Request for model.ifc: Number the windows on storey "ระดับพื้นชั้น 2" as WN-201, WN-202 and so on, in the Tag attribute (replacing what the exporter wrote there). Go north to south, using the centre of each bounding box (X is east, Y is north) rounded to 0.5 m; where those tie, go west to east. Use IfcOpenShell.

First a look at what the model holds.

```python
import ifcopenshell
import ifcopenshell.util.element
import ifcopenshell.util.placement

model = ifcopenshell.open("model.ifc")
print(model.schema)
storey = next(s for s in model.by_type("IfcBuildingStorey") if s.Name == "ระดับพื้นชั้น 2")
windows = [e for e in ifcopenshell.util.element.get_decomposition(storey) if e.is_a("IfcWindow")]
for e in sorted(windows, key=lambda e: e.id()):
    origin = ifcopenshell.util.placement.get_local_placement(e.ObjectPlacement)[:3, 3]
    print(e.id(), e.Tag, e.Name, origin.round(2) + 0.0, sep=" | ")
```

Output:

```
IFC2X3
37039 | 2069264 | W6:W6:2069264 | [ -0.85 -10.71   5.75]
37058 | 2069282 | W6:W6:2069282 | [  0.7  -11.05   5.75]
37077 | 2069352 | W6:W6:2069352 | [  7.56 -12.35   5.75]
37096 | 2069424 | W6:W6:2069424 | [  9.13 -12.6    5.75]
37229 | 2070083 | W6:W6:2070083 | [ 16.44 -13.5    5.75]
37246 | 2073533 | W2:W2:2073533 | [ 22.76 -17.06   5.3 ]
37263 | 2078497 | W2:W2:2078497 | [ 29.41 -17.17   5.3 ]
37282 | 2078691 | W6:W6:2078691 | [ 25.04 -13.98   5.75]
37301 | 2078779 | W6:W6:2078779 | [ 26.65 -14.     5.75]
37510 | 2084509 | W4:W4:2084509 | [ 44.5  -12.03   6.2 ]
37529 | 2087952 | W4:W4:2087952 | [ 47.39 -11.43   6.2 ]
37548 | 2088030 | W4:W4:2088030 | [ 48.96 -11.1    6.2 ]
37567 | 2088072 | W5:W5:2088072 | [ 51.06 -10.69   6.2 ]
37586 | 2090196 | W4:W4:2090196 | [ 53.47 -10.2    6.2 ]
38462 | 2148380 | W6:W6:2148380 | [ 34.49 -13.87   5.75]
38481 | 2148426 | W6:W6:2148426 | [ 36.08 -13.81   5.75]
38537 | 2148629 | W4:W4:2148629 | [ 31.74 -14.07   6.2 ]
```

```python
import ifcopenshell
import ifcopenshell.geom
import ifcopenshell.util.element
import ifcopenshell.util.shape

model = ifcopenshell.open("model.ifc")
settings = ifcopenshell.geom.settings()
settings.set("use-world-coords", True)


def centre(element):
    shape = ifcopenshell.geom.create_shape(settings, element)
    return ifcopenshell.util.shape.get_bbox_centroid(shape.geometry)


storey = next(s for s in model.by_type("IfcBuildingStorey") if s.Name == "ระดับพื้นชั้น 2")
windows = [e for e in ifcopenshell.util.element.get_decomposition(storey) if e.is_a("IfcWindow")]

# Insertion points can sit at a corner or the storey origin, so sort by the geometry (in metres).
centres = {e: centre(e) for e in windows}
windows.sort(key=lambda e: (-round(centres[e][1] / 0.5), centres[e][0]))

for i, e in enumerate(windows, start=1):
    number = f"WN-2{i:02d}"
    e.Tag = number
    print(e.id(), number)

model.write("model-out.ifc")
```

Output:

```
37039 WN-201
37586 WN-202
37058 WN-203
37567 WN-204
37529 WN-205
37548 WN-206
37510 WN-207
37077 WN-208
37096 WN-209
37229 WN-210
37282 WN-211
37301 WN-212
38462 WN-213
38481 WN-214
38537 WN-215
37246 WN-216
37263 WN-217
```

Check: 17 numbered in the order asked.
